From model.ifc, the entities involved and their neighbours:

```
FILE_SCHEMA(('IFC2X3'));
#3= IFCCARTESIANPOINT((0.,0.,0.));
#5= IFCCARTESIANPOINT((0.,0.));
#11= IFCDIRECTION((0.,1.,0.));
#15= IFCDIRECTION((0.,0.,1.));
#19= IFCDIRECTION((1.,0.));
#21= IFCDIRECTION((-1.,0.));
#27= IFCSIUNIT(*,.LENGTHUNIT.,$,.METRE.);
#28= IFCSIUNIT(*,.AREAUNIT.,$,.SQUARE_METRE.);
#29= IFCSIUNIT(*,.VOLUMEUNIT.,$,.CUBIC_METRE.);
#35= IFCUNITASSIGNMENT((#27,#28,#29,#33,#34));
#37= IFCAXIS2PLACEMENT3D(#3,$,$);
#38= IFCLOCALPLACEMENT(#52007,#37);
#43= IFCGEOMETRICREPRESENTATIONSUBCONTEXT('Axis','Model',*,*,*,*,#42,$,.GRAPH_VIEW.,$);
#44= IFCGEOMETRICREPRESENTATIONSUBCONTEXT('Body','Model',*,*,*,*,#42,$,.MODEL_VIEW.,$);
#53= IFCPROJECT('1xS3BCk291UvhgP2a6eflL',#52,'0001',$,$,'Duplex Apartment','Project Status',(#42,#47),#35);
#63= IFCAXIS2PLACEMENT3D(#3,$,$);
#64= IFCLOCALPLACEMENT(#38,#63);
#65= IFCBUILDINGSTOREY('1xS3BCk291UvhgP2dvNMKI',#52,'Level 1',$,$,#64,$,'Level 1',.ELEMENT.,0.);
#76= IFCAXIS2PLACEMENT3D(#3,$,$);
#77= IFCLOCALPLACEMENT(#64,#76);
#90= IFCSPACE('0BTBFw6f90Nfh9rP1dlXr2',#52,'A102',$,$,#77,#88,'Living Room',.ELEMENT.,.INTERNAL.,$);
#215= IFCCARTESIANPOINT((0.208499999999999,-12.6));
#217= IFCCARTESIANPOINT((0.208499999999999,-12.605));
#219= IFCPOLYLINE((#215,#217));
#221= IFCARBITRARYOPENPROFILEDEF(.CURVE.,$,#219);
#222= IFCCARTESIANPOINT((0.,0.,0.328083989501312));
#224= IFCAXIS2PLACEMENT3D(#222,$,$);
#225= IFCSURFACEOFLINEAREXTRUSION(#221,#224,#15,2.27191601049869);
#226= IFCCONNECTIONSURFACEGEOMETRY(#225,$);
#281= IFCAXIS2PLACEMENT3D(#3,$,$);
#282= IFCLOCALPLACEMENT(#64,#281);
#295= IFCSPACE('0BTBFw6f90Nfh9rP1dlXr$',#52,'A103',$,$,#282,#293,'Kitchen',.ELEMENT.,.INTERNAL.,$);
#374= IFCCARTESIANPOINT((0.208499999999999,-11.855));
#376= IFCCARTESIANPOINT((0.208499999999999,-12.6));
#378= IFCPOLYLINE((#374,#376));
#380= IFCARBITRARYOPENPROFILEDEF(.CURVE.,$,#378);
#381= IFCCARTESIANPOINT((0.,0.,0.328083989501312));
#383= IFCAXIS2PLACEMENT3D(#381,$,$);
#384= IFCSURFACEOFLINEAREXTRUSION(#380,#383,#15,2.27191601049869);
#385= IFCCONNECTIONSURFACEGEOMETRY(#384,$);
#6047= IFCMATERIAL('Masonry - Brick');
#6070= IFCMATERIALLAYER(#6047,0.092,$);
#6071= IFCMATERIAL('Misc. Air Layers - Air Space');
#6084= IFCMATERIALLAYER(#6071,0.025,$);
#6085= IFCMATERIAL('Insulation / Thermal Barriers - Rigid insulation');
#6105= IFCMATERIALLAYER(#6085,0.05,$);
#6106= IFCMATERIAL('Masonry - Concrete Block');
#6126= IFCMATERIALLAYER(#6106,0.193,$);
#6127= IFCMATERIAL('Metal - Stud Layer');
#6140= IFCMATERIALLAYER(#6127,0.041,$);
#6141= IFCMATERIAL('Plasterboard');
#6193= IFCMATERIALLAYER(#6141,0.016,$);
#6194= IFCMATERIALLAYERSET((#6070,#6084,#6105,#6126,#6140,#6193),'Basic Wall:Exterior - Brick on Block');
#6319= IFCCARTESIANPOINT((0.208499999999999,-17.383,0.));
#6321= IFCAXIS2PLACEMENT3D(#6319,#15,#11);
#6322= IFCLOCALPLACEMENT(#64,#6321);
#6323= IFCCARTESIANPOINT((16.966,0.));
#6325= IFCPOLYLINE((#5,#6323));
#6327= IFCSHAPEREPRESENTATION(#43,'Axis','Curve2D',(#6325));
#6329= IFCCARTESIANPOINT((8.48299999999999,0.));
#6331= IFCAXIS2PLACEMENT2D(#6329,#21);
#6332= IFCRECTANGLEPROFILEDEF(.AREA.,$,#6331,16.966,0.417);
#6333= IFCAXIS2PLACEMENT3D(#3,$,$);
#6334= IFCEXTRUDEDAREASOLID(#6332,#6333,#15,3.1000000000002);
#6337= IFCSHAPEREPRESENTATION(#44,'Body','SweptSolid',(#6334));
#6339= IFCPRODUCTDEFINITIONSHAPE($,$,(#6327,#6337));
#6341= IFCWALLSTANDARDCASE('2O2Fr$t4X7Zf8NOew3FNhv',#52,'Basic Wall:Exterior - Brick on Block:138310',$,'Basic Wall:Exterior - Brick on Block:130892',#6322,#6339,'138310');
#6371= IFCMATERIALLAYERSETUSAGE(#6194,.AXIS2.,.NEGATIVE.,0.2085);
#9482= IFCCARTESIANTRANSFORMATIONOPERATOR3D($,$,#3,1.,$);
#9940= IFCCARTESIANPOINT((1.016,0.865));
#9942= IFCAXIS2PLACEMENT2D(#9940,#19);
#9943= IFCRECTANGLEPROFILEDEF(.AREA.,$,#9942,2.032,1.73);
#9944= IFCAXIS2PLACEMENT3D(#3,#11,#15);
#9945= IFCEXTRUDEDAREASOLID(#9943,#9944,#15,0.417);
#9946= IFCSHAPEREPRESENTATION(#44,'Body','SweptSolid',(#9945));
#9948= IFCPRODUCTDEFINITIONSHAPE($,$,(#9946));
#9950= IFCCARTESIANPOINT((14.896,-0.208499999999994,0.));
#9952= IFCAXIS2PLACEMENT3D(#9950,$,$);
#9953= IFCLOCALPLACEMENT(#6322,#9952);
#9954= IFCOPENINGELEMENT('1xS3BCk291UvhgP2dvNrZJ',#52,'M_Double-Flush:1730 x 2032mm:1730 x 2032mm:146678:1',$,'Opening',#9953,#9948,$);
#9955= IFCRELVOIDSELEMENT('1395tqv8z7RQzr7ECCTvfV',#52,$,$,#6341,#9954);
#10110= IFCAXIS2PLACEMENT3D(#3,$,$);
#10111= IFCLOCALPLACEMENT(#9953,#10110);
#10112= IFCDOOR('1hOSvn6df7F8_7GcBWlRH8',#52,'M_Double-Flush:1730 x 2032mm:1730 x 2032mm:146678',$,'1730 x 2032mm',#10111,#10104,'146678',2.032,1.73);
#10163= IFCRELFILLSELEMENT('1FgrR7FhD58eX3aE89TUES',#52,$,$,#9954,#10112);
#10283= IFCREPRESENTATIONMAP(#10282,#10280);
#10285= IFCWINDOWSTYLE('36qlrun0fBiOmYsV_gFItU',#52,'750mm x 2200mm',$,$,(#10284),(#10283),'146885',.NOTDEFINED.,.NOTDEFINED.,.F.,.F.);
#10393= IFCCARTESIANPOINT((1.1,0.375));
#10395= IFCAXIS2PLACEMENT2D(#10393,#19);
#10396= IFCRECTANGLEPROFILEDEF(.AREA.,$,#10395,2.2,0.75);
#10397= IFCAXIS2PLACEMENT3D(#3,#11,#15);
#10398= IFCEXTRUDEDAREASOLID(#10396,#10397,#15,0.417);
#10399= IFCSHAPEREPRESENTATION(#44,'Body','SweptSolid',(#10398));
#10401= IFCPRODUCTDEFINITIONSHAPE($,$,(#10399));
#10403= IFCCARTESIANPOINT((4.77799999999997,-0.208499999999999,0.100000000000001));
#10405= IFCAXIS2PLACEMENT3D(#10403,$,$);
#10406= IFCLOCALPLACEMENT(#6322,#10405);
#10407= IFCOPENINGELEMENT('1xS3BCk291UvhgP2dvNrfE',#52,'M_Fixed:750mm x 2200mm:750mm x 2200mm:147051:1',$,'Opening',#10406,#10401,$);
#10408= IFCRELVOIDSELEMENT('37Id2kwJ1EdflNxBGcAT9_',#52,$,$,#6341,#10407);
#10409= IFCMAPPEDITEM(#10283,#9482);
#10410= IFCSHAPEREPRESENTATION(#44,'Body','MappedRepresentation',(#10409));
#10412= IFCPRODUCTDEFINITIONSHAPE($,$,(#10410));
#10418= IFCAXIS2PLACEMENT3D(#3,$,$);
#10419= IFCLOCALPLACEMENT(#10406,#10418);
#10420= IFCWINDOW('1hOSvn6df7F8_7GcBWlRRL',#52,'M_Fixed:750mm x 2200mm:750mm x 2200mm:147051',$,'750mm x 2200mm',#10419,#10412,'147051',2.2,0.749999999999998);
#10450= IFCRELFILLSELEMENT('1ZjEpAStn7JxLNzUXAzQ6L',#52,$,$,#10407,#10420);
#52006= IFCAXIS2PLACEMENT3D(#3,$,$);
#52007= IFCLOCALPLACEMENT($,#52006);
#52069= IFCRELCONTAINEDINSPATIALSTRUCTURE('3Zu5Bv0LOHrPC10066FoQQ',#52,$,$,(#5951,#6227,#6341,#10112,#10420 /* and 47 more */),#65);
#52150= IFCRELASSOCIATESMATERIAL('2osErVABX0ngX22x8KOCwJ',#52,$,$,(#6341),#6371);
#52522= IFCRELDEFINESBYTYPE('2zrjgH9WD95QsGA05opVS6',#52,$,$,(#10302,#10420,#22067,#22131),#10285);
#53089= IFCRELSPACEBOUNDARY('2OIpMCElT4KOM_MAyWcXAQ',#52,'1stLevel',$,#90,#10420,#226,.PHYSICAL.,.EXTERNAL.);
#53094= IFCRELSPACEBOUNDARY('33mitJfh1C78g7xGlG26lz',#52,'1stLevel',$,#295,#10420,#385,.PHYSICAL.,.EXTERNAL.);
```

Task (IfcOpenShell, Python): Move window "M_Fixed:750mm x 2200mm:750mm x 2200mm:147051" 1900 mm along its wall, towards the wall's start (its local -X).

```python
import numpy as np
import ifcopenshell
import ifcopenshell.api.geometry
import ifcopenshell.util.placement

model = ifcopenshell.open("model.ifc")

window = model.by_guid("1hOSvn6df7F8_7GcBWlRRL")
opening = window.FillsVoids[0].RelatingOpeningElement
wall = opening.VoidsElements[0].RelatingBuildingElement

wall_matrix = ifcopenshell.util.placement.get_local_placement(wall.ObjectPlacement)
shift = wall_matrix[:3, 0] * -1.9
before = ifcopenshell.util.placement.get_local_placement(window.ObjectPlacement)[:3, 3].copy()

# The window is placed relative to its opening, so it follows when the opening moves.
matrix = ifcopenshell.util.placement.get_local_placement(opening.ObjectPlacement)
matrix[:3, 3] += shift
ifcopenshell.api.geometry.edit_object_placement(
    model, product=opening, matrix=matrix, is_si=False, should_transform_children=True
)

# Space boundary surfaces are stored in each space's coordinates; move them too.
for rel in window.ProvidesBoundaries:
    if not rel.ConnectionGeometry:
        continue
    surface = rel.ConnectionGeometry.SurfaceOnRelatingElement
    space_matrix = ifcopenshell.util.placement.get_local_placement(rel.RelatingSpace.ObjectPlacement)
    point = np.array(surface.Position.Location.Coordinates) + space_matrix[:3, :3].T @ shift
    surface.Position = model.createIfcAxis2Placement3D(
        model.createIfcCartesianPoint(point.tolist()), surface.Position.Axis, surface.Position.RefDirection
    )

after = ifcopenshell.util.placement.get_local_placement(window.ObjectPlacement)[:3, 3]
print("window moved by", (after - before).round(3) + 0.0)

model.write("model_v2.ifc")
```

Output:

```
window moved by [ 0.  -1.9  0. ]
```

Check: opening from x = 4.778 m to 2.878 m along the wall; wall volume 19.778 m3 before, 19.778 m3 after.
